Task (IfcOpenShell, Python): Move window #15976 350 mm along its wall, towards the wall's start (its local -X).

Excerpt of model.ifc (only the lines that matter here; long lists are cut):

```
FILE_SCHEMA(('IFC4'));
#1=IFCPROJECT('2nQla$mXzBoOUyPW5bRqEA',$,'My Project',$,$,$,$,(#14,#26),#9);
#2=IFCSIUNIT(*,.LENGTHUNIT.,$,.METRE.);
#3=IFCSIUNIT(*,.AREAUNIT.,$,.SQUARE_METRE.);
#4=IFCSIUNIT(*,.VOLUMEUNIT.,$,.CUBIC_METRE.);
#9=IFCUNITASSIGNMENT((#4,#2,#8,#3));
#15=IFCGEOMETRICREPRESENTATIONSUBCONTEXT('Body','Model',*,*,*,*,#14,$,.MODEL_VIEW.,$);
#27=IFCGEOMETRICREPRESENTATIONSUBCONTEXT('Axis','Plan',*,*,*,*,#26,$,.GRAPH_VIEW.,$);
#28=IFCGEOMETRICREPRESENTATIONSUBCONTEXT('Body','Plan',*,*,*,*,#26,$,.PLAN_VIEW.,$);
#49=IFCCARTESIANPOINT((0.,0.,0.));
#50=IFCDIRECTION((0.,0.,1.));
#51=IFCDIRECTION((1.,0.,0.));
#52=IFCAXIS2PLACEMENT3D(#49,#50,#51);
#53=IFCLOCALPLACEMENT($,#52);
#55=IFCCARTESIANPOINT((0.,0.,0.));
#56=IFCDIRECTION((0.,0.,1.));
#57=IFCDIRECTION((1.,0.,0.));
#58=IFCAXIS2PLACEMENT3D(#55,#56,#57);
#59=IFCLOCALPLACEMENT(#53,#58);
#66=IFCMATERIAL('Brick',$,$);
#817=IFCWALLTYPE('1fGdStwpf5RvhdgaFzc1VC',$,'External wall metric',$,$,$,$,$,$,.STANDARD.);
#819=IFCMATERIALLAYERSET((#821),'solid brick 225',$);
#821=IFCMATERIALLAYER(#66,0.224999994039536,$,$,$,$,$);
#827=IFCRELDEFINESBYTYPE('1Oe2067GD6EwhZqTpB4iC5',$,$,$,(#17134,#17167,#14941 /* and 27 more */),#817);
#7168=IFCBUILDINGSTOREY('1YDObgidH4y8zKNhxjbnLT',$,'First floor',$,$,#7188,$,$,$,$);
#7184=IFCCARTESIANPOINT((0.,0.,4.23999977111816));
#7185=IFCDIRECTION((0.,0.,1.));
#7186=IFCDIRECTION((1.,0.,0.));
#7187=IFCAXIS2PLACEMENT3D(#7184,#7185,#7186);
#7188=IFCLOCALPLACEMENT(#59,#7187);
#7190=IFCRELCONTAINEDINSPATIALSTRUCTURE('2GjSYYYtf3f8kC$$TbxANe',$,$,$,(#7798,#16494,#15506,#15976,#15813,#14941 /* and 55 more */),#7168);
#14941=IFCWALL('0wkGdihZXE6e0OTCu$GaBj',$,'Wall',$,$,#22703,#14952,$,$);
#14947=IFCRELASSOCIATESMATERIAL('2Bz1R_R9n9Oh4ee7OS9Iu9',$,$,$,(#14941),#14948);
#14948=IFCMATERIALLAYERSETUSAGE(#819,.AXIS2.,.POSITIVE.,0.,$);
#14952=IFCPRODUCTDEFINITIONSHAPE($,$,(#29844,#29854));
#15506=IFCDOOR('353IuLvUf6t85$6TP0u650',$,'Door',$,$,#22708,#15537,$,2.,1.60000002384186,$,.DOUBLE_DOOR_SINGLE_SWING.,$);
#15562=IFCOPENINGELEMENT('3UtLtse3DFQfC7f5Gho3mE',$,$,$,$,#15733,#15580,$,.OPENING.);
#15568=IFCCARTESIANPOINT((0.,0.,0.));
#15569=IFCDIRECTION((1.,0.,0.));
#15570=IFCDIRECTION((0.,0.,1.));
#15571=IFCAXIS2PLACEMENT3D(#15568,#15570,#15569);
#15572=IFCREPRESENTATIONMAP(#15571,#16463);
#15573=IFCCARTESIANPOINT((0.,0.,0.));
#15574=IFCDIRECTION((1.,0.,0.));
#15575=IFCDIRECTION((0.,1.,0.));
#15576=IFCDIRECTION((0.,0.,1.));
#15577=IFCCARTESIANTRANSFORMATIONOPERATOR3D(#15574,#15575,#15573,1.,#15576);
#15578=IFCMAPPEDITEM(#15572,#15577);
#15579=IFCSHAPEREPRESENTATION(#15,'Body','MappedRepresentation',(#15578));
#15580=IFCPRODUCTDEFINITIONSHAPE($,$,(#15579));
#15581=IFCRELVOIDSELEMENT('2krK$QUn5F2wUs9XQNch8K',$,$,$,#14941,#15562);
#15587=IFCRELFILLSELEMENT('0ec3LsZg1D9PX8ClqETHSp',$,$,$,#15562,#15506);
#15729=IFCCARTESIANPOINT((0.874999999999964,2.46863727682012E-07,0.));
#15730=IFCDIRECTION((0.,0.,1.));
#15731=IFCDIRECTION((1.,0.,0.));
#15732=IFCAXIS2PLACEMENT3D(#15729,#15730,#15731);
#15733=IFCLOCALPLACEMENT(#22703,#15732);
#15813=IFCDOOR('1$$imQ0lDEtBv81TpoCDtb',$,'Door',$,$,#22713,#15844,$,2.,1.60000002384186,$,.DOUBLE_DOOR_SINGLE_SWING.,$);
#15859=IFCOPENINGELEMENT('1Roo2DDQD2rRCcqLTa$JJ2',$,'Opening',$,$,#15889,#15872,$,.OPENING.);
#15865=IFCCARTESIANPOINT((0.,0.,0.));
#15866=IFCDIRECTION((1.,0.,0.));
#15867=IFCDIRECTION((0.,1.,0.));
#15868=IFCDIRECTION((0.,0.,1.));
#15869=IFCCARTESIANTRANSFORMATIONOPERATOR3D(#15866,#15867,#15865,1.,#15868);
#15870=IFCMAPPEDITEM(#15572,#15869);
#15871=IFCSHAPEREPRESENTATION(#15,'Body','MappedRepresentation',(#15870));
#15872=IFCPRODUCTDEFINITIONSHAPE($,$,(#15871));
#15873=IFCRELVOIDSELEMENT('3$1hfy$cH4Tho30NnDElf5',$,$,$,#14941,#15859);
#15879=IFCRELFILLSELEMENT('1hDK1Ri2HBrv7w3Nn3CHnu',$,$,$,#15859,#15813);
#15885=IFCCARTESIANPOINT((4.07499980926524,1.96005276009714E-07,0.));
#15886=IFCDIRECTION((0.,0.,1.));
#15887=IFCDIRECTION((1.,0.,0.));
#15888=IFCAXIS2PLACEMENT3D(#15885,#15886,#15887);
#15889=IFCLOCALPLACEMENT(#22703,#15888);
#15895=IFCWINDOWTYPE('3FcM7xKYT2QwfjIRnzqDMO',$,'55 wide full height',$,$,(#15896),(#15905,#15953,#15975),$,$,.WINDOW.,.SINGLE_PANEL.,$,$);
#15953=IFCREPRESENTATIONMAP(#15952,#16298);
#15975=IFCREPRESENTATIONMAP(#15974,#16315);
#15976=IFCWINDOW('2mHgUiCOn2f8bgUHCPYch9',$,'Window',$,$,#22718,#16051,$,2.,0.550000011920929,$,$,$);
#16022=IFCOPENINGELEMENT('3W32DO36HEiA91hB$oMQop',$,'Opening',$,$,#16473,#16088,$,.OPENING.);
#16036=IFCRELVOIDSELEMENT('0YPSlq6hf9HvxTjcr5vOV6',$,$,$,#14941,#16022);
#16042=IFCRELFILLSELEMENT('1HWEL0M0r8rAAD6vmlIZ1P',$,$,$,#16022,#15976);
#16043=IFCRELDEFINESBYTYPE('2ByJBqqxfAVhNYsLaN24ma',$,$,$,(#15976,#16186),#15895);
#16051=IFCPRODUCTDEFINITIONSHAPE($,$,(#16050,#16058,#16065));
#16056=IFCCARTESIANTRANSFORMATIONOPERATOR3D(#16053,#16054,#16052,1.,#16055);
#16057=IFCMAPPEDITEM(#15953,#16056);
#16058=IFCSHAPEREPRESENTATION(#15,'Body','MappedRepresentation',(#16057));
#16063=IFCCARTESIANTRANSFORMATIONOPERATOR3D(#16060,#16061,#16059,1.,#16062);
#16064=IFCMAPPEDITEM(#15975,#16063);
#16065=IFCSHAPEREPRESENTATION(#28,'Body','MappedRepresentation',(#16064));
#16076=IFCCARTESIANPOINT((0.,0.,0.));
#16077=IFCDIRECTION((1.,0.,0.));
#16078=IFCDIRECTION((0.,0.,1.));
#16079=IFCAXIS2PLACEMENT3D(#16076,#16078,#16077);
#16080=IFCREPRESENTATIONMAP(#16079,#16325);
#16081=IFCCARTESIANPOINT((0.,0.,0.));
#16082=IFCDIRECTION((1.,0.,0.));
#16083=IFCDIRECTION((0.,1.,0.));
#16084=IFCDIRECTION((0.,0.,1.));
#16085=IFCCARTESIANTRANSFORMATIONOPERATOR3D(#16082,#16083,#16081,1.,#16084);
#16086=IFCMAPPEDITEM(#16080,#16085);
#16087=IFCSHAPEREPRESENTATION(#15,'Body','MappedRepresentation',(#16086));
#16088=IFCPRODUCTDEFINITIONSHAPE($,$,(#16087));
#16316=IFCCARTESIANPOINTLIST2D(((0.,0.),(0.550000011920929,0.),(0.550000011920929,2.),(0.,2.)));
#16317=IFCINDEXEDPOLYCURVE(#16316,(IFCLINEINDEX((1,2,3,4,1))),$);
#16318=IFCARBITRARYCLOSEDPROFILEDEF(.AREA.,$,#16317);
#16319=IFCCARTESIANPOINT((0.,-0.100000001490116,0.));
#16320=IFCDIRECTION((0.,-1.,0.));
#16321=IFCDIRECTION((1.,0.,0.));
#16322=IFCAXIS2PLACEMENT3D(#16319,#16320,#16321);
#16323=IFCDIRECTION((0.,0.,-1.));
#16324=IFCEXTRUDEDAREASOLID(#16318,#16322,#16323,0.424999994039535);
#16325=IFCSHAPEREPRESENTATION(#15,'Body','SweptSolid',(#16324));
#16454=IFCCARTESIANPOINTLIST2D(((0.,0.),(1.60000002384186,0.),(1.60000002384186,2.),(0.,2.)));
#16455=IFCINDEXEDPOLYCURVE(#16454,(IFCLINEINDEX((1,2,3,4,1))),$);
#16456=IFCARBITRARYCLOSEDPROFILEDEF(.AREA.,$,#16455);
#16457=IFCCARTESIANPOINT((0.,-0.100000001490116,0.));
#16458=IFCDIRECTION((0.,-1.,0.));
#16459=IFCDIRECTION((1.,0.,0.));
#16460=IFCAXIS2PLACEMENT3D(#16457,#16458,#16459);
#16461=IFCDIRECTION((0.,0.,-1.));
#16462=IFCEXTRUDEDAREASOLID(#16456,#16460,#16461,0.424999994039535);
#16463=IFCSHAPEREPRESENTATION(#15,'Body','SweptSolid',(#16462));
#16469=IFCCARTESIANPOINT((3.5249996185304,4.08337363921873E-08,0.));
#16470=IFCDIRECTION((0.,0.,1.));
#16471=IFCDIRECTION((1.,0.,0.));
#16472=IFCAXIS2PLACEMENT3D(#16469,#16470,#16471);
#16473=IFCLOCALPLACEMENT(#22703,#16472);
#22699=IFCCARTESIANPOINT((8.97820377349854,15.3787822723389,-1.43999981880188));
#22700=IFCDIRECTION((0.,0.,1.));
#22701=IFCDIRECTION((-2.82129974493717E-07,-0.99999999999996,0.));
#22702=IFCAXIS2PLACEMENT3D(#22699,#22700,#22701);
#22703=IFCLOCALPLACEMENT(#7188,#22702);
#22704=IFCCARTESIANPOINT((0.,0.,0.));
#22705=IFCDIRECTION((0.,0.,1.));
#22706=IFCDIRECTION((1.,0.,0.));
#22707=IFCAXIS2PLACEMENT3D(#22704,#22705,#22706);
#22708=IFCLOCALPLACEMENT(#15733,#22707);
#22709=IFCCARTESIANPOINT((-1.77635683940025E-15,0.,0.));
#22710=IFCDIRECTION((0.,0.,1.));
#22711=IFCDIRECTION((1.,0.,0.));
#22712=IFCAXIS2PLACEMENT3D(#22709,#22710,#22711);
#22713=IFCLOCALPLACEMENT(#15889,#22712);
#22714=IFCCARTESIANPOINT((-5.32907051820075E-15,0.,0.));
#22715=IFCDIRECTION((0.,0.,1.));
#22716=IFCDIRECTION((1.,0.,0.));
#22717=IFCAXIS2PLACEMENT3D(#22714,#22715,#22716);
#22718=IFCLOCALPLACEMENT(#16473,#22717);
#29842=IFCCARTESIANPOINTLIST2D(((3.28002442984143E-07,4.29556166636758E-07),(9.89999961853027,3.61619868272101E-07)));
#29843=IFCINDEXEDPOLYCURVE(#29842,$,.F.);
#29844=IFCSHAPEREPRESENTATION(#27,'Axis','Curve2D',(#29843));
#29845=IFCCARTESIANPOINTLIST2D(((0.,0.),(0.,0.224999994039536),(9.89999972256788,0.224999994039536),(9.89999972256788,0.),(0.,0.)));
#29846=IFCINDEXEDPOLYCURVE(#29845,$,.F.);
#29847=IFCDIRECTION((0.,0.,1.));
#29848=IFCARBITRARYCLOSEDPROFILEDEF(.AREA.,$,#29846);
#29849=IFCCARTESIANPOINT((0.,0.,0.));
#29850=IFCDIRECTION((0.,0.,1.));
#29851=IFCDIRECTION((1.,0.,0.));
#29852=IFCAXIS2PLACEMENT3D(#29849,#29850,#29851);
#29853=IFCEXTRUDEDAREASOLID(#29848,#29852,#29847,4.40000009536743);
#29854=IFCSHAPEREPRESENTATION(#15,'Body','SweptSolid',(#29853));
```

```python
import ifcopenshell
import ifcopenshell.api.geometry
import ifcopenshell.util.placement

model = ifcopenshell.open("model.ifc")

window = model.by_guid("2mHgUiCOn2f8bgUHCPYch9")
opening = window.FillsVoids[0].RelatingOpeningElement
wall = opening.VoidsElements[0].RelatingBuildingElement

wall_matrix = ifcopenshell.util.placement.get_local_placement(wall.ObjectPlacement)
shift = wall_matrix[:3, 0] * -0.35
before = ifcopenshell.util.placement.get_local_placement(window.ObjectPlacement)[:3, 3].copy()

# The window is placed relative to its opening, so it follows when the opening moves.
matrix = ifcopenshell.util.placement.get_local_placement(opening.ObjectPlacement)
matrix[:3, 3] += shift
ifcopenshell.api.geometry.edit_object_placement(
    model, product=opening, matrix=matrix, is_si=False, should_transform_children=True
)

after = ifcopenshell.util.placement.get_local_placement(window.ObjectPlacement)[:3, 3]
print("window moved by", (after - before).round(3) + 0.0)

model.write("model_updated.ifc")
```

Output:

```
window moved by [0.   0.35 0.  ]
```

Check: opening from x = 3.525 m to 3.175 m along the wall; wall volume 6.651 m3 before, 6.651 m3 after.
